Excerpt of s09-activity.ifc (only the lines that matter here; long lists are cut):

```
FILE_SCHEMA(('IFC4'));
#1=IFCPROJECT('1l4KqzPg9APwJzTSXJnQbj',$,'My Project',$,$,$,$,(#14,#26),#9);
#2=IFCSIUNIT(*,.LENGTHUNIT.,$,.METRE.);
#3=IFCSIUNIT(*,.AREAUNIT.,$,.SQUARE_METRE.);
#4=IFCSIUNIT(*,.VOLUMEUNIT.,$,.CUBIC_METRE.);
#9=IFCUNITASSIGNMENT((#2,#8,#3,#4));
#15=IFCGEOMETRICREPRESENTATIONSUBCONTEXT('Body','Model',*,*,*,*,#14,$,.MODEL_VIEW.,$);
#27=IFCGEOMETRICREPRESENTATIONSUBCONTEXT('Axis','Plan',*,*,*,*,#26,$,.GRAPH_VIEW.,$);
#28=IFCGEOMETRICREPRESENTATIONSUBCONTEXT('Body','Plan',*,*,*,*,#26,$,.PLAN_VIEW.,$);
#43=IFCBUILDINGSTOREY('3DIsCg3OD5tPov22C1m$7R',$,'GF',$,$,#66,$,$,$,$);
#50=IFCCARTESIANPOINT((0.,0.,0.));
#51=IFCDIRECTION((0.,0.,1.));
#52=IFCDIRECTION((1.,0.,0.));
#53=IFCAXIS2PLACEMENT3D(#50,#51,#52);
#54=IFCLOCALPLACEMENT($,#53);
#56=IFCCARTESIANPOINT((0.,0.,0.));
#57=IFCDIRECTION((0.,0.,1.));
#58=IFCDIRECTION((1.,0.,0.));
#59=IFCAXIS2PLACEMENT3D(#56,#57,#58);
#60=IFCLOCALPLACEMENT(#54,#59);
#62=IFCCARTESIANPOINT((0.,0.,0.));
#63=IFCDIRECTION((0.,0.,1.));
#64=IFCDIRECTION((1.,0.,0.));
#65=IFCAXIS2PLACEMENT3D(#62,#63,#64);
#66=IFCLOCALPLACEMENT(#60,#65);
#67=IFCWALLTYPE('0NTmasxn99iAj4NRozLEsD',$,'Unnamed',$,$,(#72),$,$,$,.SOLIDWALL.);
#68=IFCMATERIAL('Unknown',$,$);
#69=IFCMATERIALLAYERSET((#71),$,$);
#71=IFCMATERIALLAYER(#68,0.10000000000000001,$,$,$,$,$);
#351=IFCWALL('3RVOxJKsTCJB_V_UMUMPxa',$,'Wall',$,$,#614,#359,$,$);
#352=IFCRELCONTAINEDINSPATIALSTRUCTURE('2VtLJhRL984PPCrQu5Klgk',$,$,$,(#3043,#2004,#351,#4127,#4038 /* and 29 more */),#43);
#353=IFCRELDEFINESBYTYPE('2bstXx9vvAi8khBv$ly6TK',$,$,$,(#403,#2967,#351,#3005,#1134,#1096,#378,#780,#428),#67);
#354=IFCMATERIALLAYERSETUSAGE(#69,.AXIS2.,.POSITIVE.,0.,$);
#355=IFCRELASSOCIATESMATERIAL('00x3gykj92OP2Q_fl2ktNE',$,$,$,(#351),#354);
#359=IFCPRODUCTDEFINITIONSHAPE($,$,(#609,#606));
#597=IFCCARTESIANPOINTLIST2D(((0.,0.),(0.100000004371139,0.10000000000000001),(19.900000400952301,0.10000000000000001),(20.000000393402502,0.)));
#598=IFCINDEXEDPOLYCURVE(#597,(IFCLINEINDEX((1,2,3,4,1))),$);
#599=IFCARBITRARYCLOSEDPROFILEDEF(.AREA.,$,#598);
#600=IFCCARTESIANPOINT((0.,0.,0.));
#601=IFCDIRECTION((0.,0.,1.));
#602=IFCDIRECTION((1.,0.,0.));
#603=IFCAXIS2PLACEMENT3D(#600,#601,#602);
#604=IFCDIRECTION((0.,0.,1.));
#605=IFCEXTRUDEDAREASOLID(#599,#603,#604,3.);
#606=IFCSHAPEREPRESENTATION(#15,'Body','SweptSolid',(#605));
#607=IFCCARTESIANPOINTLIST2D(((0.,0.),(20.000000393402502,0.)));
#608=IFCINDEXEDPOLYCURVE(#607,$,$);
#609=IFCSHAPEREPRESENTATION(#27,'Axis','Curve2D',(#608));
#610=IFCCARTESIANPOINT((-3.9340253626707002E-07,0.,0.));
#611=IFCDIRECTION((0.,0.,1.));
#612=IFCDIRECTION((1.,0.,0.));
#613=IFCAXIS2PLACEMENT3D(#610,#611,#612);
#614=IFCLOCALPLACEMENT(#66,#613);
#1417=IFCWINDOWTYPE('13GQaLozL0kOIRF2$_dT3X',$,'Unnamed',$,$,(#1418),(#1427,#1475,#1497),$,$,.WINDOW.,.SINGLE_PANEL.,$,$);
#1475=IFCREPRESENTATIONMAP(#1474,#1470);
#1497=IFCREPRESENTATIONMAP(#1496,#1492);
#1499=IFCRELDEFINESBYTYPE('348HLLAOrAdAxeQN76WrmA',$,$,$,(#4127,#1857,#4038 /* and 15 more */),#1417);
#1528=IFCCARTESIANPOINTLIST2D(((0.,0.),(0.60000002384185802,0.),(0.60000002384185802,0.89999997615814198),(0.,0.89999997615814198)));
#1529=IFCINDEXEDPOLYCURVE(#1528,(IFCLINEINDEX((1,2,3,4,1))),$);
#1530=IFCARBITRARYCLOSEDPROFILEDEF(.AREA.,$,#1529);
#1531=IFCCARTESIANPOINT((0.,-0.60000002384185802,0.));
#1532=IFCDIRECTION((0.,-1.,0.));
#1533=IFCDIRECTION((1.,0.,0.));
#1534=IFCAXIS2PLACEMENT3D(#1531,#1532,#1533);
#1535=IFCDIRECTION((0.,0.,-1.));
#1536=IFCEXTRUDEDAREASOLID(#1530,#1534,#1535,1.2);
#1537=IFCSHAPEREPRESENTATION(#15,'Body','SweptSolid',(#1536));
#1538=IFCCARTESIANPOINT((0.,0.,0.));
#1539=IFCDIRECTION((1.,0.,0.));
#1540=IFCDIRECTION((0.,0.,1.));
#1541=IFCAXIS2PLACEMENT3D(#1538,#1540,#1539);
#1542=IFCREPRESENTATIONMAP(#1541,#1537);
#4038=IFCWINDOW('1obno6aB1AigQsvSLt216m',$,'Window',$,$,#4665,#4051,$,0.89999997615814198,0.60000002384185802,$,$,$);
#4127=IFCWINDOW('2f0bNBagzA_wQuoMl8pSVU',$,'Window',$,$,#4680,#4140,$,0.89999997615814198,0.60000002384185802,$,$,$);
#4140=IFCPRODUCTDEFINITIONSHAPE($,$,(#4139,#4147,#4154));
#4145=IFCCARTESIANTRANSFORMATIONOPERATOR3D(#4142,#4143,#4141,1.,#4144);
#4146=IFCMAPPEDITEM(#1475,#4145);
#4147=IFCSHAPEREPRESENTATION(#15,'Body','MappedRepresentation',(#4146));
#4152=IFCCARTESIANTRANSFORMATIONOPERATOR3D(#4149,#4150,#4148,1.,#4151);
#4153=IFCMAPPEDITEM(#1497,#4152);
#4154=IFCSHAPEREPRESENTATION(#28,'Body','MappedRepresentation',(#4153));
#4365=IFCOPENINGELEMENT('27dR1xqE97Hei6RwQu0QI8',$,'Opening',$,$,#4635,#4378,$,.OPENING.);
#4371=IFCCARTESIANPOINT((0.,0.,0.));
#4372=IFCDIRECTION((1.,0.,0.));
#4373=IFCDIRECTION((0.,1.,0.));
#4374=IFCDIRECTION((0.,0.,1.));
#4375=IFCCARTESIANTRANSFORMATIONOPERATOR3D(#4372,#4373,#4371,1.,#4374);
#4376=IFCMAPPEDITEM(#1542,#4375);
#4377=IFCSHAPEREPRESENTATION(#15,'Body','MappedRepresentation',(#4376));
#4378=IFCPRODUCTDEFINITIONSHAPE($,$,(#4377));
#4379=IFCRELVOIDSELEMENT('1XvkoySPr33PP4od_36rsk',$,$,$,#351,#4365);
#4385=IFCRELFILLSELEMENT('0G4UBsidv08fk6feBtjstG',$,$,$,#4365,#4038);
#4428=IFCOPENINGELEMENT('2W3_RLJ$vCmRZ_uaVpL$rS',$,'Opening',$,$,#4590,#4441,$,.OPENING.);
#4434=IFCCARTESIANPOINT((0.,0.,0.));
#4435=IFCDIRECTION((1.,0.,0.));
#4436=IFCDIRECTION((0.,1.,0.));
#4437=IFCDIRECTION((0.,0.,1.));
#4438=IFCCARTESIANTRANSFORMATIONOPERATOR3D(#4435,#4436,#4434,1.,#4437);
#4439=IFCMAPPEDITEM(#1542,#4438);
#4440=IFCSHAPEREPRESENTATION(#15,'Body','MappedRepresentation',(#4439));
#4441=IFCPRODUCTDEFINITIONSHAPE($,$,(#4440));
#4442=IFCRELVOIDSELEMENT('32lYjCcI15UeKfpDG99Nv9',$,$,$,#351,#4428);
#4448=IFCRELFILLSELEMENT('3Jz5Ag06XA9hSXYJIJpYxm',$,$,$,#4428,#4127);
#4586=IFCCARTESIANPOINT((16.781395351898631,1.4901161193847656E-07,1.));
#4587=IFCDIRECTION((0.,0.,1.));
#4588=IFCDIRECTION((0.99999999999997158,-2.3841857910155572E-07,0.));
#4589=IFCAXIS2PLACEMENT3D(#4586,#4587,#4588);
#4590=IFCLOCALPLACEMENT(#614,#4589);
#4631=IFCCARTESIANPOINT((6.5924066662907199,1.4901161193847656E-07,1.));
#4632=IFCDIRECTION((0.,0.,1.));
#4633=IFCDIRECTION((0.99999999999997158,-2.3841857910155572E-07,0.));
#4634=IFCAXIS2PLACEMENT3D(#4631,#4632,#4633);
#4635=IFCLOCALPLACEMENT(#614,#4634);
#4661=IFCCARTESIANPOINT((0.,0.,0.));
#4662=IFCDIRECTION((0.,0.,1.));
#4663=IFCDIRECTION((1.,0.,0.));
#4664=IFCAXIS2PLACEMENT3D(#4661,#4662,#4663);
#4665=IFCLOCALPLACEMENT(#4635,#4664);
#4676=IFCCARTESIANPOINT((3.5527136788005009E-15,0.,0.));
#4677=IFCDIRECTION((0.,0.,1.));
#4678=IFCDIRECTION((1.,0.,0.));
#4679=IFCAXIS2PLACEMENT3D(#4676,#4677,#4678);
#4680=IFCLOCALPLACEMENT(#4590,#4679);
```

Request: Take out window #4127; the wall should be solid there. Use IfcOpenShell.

```python
import ifcopenshell
import ifcopenshell.api.feature
import ifcopenshell.api.root
import ifcopenshell.geom
import ifcopenshell.util.shape

model = ifcopenshell.open("s09-activity.ifc")
settings = ifcopenshell.geom.settings()


def volume(element):
    """Net volume in cubic metres, openings subtracted."""
    shape = ifcopenshell.geom.create_shape(settings, element)
    return ifcopenshell.util.shape.get_volume(shape.geometry)


window = model.by_guid("2f0bNBagzA_wQuoMl8pSVU")
opening = window.FillsVoids[0].RelatingOpeningElement
wall = opening.VoidsElements[0].RelatingBuildingElement
before = volume(wall)

ifcopenshell.api.root.remove_product(model, product=window)
ifcopenshell.api.feature.remove_feature(model, feature=opening)

after = volume(wall)

print(f"wall volume {before:.3f} -> {after:.3f} m3")

model.write("s09-activity_updated.ifc")
```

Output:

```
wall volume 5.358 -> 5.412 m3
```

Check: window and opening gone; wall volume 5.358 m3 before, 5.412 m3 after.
